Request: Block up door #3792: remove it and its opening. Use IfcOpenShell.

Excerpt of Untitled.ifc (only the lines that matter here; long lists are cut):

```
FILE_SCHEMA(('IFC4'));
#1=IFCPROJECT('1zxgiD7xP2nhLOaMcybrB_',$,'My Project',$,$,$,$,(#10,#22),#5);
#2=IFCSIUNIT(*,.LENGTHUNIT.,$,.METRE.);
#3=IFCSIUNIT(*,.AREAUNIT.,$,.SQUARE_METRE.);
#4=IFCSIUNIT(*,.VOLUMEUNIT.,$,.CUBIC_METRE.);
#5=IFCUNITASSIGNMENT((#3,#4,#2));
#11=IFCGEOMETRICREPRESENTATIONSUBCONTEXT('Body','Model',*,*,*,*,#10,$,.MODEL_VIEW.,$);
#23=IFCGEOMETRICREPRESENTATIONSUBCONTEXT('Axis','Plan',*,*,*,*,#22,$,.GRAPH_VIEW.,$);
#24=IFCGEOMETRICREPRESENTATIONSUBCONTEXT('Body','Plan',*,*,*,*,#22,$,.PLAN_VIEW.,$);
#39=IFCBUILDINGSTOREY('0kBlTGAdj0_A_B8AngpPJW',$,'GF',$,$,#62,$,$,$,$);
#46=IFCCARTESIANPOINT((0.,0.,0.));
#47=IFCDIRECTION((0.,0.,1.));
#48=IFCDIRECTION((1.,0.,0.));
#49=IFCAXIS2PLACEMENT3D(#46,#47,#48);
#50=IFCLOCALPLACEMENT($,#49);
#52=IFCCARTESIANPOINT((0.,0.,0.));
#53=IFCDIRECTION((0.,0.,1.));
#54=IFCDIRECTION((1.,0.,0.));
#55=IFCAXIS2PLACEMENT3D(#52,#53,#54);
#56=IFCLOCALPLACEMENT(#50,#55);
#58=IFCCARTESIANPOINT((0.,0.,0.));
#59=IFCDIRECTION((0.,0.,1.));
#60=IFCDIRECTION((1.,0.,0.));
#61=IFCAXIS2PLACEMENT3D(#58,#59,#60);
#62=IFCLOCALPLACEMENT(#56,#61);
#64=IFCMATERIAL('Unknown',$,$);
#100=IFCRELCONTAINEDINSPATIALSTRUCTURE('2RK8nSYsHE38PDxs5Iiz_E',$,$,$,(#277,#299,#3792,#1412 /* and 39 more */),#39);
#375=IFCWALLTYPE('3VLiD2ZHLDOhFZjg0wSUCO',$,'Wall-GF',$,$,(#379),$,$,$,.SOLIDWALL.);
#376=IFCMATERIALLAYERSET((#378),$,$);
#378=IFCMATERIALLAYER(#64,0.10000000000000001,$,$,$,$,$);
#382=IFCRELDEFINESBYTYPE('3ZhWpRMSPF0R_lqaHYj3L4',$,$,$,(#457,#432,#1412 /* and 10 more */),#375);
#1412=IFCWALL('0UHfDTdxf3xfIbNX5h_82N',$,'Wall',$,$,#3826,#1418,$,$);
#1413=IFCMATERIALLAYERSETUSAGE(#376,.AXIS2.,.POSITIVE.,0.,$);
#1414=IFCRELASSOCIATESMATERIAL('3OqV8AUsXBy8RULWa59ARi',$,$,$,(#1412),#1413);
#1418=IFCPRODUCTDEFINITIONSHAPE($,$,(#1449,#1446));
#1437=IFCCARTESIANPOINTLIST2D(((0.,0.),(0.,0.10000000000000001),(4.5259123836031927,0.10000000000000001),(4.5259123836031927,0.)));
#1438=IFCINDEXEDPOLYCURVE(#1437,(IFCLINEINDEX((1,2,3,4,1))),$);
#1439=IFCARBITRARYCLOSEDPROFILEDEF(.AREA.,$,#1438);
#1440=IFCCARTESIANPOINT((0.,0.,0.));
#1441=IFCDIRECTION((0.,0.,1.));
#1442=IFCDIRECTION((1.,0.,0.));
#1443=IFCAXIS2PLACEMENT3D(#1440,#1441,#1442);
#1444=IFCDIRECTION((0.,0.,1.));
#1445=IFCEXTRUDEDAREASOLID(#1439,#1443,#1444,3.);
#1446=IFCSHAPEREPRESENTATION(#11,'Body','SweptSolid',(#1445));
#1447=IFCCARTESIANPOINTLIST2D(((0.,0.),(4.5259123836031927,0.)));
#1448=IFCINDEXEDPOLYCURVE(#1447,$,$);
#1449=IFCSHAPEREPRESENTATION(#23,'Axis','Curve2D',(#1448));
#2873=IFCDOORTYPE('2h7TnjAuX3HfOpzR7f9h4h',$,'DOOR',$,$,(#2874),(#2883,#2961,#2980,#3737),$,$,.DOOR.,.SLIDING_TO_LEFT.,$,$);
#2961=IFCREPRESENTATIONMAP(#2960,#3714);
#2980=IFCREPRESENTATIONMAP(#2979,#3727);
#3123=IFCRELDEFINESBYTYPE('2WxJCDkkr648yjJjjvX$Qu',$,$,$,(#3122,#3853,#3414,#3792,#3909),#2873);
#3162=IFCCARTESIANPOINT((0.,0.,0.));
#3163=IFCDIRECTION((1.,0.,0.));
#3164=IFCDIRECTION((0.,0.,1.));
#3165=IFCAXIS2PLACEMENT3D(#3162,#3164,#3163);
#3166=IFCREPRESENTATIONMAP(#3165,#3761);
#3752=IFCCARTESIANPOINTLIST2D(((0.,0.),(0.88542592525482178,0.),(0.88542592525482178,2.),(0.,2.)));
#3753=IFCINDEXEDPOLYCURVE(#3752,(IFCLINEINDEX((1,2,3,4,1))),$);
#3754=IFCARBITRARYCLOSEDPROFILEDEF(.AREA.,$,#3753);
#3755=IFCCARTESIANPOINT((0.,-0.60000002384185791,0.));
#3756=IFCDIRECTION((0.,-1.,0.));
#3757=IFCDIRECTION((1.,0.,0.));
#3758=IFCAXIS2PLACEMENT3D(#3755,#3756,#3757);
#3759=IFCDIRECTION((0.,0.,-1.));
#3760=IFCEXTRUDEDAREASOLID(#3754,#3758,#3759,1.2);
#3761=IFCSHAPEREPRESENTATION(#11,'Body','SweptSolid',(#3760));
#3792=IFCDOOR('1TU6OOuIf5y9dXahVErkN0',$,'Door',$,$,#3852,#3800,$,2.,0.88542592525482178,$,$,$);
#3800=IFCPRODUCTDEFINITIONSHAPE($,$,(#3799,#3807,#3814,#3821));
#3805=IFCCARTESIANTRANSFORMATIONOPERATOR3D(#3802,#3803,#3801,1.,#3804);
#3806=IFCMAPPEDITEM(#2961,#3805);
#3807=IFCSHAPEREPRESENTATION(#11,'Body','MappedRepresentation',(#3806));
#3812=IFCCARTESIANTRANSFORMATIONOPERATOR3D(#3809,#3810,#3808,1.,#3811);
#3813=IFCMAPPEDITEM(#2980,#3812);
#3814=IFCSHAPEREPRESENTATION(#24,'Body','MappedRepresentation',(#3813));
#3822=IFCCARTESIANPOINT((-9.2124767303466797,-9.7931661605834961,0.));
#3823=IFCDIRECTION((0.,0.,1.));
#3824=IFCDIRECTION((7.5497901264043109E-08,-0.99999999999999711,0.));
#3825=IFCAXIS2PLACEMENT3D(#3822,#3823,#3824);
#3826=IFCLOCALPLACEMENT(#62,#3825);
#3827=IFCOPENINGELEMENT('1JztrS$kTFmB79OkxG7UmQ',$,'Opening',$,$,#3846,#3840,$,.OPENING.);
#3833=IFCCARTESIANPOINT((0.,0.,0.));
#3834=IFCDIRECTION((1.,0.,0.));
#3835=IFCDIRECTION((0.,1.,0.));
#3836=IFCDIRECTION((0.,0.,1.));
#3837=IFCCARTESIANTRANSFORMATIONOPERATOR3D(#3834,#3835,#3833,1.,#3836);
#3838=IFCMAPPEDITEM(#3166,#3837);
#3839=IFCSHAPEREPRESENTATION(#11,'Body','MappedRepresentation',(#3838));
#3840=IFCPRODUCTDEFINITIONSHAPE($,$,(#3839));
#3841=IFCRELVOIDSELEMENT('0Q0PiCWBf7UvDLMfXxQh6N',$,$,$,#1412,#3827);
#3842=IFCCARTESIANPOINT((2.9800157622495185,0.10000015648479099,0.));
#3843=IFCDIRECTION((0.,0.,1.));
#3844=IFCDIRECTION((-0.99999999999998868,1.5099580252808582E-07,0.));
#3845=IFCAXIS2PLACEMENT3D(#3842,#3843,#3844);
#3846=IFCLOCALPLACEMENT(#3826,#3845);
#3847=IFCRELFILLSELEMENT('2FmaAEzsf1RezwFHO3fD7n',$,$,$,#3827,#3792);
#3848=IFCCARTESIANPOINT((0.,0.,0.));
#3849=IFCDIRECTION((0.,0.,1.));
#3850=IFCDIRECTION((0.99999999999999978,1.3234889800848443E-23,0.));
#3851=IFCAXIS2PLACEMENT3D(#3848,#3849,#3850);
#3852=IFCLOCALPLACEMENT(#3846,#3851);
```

```python
import ifcopenshell
import ifcopenshell.api.feature
import ifcopenshell.api.root
import ifcopenshell.geom
import ifcopenshell.util.shape

model = ifcopenshell.open("Untitled.ifc")
settings = ifcopenshell.geom.settings()


def volume(element):
    """Net volume in cubic metres, openings subtracted."""
    shape = ifcopenshell.geom.create_shape(settings, element)
    return ifcopenshell.util.shape.get_volume(shape.geometry)


door = model.by_guid("1TU6OOuIf5y9dXahVErkN0")
opening = door.FillsVoids[0].RelatingOpeningElement
wall = opening.VoidsElements[0].RelatingBuildingElement
before = volume(wall)

ifcopenshell.api.root.remove_product(model, product=door)
ifcopenshell.api.feature.remove_feature(model, feature=opening)

after = volume(wall)

print(f"wall volume {before:.3f} -> {after:.3f} m3")

model.write("Untitled_updated.ifc")
```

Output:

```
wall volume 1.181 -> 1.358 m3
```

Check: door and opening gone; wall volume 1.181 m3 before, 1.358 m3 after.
